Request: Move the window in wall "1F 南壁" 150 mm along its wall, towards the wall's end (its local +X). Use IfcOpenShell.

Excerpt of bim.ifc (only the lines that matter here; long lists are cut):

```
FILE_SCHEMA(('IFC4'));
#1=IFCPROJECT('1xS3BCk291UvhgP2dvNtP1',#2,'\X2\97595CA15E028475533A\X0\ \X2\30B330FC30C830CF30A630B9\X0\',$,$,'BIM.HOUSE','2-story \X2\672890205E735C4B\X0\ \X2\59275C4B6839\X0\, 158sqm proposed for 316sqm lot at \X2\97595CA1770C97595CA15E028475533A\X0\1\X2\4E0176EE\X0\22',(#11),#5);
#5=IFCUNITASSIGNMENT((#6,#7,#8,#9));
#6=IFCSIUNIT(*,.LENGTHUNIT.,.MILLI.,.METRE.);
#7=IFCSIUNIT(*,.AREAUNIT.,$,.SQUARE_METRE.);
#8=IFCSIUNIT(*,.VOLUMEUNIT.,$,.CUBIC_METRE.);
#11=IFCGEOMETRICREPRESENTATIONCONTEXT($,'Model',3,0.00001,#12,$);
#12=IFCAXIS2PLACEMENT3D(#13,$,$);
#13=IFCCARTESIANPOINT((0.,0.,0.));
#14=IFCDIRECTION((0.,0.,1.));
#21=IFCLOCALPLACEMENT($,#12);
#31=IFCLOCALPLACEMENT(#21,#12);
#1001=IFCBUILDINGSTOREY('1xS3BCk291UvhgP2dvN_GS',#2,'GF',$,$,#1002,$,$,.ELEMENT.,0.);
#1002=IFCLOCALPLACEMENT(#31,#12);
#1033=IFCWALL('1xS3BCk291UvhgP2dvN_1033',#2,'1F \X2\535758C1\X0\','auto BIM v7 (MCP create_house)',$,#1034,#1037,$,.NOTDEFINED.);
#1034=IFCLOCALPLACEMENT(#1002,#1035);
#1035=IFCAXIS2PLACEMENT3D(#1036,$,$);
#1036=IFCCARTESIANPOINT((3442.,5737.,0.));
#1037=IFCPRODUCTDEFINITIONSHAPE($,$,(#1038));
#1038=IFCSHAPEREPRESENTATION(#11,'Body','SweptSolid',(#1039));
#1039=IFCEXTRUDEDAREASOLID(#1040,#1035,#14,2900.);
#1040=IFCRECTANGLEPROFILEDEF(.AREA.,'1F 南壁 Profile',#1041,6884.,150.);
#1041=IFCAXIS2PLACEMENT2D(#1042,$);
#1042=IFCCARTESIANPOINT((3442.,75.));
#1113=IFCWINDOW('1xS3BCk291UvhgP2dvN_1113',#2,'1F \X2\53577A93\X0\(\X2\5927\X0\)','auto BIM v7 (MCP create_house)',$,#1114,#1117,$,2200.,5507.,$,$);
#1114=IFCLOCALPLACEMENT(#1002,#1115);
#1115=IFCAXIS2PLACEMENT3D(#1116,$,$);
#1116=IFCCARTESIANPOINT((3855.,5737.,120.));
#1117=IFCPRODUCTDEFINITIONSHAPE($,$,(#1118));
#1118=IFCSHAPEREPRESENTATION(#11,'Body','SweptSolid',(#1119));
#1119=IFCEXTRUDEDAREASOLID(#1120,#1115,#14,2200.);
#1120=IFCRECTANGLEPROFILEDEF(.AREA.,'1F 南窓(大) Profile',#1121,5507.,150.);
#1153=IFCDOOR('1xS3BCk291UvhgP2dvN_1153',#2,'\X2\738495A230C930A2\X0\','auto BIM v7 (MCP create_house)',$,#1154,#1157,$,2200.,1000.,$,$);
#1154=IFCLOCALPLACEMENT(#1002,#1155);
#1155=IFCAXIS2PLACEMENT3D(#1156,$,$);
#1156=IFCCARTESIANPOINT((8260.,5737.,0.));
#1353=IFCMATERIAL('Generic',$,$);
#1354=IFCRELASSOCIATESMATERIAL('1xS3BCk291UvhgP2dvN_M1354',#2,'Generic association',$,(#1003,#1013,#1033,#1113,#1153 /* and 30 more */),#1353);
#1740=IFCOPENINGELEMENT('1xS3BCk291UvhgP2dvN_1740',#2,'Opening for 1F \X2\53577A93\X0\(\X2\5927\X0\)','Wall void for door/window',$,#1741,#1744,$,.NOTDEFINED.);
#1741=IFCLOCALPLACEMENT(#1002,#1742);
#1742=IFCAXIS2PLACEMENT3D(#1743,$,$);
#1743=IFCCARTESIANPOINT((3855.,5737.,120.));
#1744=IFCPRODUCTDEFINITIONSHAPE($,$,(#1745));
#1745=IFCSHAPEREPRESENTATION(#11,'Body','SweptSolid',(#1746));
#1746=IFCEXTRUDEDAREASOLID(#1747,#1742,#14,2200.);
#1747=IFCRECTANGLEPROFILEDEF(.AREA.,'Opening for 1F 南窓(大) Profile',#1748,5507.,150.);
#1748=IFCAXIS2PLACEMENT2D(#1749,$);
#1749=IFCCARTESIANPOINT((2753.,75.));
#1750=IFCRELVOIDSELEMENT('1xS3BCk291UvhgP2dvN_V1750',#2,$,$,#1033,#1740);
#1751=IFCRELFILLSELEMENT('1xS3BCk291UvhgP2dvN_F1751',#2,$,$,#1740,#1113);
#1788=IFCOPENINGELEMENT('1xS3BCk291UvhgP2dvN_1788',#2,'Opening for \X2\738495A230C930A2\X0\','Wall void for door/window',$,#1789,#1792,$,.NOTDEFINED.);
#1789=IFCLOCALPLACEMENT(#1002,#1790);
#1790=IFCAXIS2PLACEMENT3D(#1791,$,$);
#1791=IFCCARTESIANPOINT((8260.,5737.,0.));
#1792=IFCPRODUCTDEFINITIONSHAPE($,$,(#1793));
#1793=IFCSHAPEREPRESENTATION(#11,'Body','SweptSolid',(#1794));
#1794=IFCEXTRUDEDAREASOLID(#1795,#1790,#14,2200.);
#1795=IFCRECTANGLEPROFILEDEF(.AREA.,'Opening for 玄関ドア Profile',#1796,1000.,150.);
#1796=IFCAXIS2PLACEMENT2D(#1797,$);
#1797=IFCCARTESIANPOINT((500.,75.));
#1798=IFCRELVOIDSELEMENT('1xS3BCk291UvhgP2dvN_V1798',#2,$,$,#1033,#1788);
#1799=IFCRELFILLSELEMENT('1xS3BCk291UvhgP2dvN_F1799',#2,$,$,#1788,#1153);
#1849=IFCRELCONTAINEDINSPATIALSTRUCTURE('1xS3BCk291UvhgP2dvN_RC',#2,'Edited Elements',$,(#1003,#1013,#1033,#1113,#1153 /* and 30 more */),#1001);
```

```python
import ifcopenshell
import ifcopenshell.api.geometry
import ifcopenshell.util.placement

model = ifcopenshell.open("bim.ifc")

window = model.by_id(1113)
opening = window.FillsVoids[0].RelatingOpeningElement
wall = opening.VoidsElements[0].RelatingBuildingElement

wall_matrix = ifcopenshell.util.placement.get_local_placement(wall.ObjectPlacement)
shift = wall_matrix[:3, 0] * 150.0
before = ifcopenshell.util.placement.get_local_placement(window.ObjectPlacement)[:3, 3].copy()

# The window is not placed relative to its opening, so move both.
for product in (opening, window):
    matrix = ifcopenshell.util.placement.get_local_placement(product.ObjectPlacement)
    matrix[:3, 3] += shift
    ifcopenshell.api.geometry.edit_object_placement(model, product=product, matrix=matrix, is_si=False)

after = ifcopenshell.util.placement.get_local_placement(window.ObjectPlacement)[:3, 3]
print("window moved by", (after - before).round(3) + 0.0)

model.write("bim_updated.ifc")
```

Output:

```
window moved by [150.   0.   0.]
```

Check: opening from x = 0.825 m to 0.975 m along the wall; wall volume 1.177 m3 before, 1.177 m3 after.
